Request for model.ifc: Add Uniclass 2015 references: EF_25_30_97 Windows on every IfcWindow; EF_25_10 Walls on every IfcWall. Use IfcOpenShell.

First a look at what the model holds.

```python
import ifcopenshell

model = ifcopenshell.open("model.ifc")
print(model.schema)
print("classifications:", [c.Name for c in model.by_type("IfcClassification")])
for ifc_class in ("IfcDoor", "IfcRoof", "IfcStair", "IfcWall", "IfcWindow"):
    print(ifc_class, len(model.by_type(ifc_class)))
```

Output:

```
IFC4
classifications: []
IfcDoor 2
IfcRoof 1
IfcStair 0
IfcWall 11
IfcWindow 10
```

```python
import ifcopenshell
import ifcopenshell.api.classification

model = ifcopenshell.open("model.ifc")

system = ifcopenshell.api.classification.add_classification(model, classification="Uniclass 2015")

codes = {
    "IfcWindow": ("EF_25_30_97", "Windows"),
    "IfcWall": ("EF_25_10", "Walls"),
}
for ifc_class, (code, name) in codes.items():
    products = model.by_type(ifc_class)
    ifcopenshell.api.classification.add_reference(
        model, products=products, classification=system, identification=code, name=name
    )
    print(code, len(products))

model.write("model_rev.ifc")
```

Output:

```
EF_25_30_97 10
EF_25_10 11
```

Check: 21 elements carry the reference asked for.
